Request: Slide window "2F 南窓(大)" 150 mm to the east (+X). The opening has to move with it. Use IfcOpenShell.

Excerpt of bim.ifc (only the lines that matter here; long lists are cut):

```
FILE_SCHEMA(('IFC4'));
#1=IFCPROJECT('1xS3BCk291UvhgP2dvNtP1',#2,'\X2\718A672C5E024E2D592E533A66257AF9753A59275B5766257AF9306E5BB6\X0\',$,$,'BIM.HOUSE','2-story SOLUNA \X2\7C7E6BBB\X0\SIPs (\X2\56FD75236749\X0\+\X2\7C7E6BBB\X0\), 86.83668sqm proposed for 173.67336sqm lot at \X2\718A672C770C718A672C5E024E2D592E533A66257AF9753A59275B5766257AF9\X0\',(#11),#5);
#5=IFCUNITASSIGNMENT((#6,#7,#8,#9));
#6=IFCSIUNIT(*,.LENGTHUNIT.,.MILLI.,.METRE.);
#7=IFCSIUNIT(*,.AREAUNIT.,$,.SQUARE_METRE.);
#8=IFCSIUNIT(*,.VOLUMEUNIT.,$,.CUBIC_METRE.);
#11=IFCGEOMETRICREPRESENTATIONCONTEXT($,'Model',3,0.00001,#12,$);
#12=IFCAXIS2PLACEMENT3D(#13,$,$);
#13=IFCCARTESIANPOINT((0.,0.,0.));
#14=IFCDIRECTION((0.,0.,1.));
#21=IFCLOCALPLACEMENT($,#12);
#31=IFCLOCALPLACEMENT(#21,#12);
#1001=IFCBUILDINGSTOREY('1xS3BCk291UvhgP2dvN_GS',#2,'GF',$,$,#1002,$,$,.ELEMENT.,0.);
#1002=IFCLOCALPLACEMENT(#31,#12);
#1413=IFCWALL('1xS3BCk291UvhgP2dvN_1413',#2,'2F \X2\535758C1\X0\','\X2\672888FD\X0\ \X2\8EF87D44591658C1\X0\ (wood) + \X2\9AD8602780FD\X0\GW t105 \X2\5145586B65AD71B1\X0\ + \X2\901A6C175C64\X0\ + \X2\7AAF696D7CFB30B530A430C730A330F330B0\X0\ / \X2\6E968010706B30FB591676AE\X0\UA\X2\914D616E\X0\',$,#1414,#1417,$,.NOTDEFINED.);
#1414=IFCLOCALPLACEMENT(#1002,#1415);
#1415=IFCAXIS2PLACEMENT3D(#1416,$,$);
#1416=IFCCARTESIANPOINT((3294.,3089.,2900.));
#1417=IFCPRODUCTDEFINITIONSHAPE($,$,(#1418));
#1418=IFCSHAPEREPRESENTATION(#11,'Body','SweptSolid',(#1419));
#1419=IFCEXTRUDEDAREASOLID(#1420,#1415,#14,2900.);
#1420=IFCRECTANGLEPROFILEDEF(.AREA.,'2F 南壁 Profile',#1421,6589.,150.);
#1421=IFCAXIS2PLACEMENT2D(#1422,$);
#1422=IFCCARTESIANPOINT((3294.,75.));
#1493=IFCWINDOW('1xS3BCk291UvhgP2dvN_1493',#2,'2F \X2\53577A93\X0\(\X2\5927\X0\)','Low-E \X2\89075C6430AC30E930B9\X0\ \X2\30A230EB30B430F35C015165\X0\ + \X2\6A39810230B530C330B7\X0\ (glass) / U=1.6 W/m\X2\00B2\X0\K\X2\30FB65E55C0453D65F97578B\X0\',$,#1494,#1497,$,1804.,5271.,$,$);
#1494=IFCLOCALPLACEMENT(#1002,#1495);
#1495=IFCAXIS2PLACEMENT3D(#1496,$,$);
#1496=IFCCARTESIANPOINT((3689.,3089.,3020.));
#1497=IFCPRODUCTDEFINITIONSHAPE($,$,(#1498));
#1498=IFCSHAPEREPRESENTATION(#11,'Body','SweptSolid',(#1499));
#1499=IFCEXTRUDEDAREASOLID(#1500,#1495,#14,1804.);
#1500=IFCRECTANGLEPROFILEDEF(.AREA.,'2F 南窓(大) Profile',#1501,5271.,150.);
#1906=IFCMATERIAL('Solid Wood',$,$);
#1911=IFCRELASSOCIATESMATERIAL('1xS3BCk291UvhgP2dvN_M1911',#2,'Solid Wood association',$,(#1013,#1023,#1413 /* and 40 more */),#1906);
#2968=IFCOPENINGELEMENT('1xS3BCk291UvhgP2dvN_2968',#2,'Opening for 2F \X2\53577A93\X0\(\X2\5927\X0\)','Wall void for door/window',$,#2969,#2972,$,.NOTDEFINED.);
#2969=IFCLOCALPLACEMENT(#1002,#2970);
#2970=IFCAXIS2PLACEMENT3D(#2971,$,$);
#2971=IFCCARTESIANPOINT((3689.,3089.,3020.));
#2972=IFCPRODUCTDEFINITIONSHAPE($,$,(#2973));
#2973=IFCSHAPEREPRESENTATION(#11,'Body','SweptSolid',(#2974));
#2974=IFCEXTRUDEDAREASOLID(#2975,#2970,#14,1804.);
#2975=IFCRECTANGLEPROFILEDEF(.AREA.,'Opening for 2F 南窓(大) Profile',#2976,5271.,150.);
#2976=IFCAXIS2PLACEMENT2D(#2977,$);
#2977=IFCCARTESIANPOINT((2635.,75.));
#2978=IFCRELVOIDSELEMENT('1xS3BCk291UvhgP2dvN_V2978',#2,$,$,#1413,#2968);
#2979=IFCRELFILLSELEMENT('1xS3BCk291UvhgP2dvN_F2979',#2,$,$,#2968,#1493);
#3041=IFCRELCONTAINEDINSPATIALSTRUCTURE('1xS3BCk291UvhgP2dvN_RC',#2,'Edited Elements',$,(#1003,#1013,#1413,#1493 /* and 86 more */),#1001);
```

```python
import ifcopenshell
import ifcopenshell.api.geometry
import ifcopenshell.util.placement
import ifcopenshell.util.unit

model = ifcopenshell.open("bim.ifc")
unit_scale = ifcopenshell.util.unit.calculate_unit_scale(model)

window = model.by_id(1493)
opening = window.FillsVoids[0].RelatingOpeningElement
wall = opening.VoidsElements[0].RelatingBuildingElement

wall_matrix = ifcopenshell.util.placement.get_local_placement(wall.ObjectPlacement)
shift = wall_matrix[:3, 0] * 0.15 / unit_scale
before = ifcopenshell.util.placement.get_local_placement(window.ObjectPlacement)[:3, 3].copy()

# The window is not placed relative to its opening, so move both.
for product in (opening, window):
    matrix = ifcopenshell.util.placement.get_local_placement(product.ObjectPlacement)
    matrix[:3, 3] += shift
    ifcopenshell.api.geometry.edit_object_placement(model, product=product, matrix=matrix, is_si=False)

after = ifcopenshell.util.placement.get_local_placement(window.ObjectPlacement)[:3, 3]
print("window moved by", (after - before).round(3) + 0.0)

model.write("bim_edited.ifc")
```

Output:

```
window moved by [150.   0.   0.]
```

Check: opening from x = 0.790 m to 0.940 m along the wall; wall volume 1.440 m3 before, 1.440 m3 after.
